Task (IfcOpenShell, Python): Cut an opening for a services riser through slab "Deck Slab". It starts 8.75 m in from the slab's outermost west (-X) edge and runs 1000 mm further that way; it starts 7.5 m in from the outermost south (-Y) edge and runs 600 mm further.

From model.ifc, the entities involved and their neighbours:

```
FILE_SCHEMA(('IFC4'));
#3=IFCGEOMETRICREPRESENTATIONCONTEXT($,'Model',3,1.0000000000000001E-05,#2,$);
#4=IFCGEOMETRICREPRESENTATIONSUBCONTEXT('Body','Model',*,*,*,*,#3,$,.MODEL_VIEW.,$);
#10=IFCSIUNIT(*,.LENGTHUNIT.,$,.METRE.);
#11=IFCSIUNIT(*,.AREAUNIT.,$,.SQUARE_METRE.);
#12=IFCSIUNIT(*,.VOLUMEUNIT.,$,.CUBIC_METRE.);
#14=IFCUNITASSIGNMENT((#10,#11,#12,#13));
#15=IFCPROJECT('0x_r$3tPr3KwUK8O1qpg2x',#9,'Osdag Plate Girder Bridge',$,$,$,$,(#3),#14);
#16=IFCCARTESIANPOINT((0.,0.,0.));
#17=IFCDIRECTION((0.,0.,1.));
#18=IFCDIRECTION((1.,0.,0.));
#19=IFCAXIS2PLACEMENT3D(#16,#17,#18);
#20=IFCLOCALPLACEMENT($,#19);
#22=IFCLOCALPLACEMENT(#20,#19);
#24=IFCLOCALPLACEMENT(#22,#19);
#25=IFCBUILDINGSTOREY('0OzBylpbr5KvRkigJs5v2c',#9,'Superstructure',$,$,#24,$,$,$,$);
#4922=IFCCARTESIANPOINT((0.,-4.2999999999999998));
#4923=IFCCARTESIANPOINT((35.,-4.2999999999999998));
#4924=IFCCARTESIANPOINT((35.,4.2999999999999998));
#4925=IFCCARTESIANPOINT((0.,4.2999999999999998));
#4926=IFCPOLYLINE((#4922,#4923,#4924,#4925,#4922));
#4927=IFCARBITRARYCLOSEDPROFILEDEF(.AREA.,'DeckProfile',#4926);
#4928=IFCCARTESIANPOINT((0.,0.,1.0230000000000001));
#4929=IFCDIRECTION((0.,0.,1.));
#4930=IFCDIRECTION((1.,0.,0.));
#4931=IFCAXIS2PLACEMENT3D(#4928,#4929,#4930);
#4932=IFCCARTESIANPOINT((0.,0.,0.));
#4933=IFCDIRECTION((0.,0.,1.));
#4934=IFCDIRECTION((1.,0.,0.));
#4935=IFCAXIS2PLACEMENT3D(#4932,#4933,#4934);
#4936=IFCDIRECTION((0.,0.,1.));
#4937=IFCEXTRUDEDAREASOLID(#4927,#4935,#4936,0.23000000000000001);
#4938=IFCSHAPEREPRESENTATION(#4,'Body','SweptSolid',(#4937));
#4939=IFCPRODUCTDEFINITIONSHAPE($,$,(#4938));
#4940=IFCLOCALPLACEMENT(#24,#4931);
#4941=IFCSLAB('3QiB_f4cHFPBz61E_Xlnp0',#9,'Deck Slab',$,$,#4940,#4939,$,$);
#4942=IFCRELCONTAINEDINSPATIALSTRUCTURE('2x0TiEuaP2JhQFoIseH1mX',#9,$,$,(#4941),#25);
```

```python
import numpy as np
import ifcopenshell
import ifcopenshell.api.feature
import ifcopenshell.api.geometry
import ifcopenshell.api.root
import ifcopenshell.geom
import ifcopenshell.util.placement
import ifcopenshell.util.representation
import ifcopenshell.util.shape
import ifcopenshell.util.unit

model = ifcopenshell.open("model.ifc")
unit_scale = ifcopenshell.util.unit.calculate_unit_scale(model)
settings = ifcopenshell.geom.settings()


def volume(element):
    """Net volume in cubic metres, openings subtracted."""
    shape = ifcopenshell.geom.create_shape(settings, element)
    return ifcopenshell.util.shape.get_volume(shape.geometry)


slab = model.by_guid("3QiB_f4cHFPBz61E_Xlnp0")
before = volume(slab)

# Extent in the slab's own axes, in metres. The edges named are its -X and -Y sides.
slab_shape = ifcopenshell.geom.create_shape(settings, slab)
vertices = ifcopenshell.util.shape.get_vertices(slab_shape.geometry)
x_min, y_min, bottom = vertices.min(axis=0)
top = vertices[:, 2].max()

opening = ifcopenshell.api.root.create_entity(model, ifc_class="IfcOpeningElement", name="Services riser opening", predefined_type="OPENING")
context = ifcopenshell.util.representation.get_context(model, "Model", "Body", "MODEL_VIEW")
width, depth = 1, 0.6
outline = [(0.0, 0.0), (width, 0.0), (width, depth), (0.0, depth), (0.0, 0.0)]
# Overshoot both faces by 50 mm so the cut is clean.
shape = ifcopenshell.api.geometry.add_slab_representation(
    model, context=context, depth=top - bottom + 0.1, polyline=outline
)
ifcopenshell.api.geometry.assign_representation(model, product=opening, representation=shape)

matrix = ifcopenshell.util.placement.get_local_placement(slab.ObjectPlacement)
matrix[:, 3] = matrix @ np.append(np.array([x_min + 8.75, y_min + 7.5, bottom - 0.05]) / unit_scale, 1.0)
ifcopenshell.api.geometry.edit_object_placement(model, product=opening, matrix=matrix, is_si=False)
ifcopenshell.api.feature.add_feature(model, feature=opening, element=slab)

after = volume(slab)

print(f"slab volume {before:.3f} -> {after:.3f} m3")

model.write("model_edited.ifc")
```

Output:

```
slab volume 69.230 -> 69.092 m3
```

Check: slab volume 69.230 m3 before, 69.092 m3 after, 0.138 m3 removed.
